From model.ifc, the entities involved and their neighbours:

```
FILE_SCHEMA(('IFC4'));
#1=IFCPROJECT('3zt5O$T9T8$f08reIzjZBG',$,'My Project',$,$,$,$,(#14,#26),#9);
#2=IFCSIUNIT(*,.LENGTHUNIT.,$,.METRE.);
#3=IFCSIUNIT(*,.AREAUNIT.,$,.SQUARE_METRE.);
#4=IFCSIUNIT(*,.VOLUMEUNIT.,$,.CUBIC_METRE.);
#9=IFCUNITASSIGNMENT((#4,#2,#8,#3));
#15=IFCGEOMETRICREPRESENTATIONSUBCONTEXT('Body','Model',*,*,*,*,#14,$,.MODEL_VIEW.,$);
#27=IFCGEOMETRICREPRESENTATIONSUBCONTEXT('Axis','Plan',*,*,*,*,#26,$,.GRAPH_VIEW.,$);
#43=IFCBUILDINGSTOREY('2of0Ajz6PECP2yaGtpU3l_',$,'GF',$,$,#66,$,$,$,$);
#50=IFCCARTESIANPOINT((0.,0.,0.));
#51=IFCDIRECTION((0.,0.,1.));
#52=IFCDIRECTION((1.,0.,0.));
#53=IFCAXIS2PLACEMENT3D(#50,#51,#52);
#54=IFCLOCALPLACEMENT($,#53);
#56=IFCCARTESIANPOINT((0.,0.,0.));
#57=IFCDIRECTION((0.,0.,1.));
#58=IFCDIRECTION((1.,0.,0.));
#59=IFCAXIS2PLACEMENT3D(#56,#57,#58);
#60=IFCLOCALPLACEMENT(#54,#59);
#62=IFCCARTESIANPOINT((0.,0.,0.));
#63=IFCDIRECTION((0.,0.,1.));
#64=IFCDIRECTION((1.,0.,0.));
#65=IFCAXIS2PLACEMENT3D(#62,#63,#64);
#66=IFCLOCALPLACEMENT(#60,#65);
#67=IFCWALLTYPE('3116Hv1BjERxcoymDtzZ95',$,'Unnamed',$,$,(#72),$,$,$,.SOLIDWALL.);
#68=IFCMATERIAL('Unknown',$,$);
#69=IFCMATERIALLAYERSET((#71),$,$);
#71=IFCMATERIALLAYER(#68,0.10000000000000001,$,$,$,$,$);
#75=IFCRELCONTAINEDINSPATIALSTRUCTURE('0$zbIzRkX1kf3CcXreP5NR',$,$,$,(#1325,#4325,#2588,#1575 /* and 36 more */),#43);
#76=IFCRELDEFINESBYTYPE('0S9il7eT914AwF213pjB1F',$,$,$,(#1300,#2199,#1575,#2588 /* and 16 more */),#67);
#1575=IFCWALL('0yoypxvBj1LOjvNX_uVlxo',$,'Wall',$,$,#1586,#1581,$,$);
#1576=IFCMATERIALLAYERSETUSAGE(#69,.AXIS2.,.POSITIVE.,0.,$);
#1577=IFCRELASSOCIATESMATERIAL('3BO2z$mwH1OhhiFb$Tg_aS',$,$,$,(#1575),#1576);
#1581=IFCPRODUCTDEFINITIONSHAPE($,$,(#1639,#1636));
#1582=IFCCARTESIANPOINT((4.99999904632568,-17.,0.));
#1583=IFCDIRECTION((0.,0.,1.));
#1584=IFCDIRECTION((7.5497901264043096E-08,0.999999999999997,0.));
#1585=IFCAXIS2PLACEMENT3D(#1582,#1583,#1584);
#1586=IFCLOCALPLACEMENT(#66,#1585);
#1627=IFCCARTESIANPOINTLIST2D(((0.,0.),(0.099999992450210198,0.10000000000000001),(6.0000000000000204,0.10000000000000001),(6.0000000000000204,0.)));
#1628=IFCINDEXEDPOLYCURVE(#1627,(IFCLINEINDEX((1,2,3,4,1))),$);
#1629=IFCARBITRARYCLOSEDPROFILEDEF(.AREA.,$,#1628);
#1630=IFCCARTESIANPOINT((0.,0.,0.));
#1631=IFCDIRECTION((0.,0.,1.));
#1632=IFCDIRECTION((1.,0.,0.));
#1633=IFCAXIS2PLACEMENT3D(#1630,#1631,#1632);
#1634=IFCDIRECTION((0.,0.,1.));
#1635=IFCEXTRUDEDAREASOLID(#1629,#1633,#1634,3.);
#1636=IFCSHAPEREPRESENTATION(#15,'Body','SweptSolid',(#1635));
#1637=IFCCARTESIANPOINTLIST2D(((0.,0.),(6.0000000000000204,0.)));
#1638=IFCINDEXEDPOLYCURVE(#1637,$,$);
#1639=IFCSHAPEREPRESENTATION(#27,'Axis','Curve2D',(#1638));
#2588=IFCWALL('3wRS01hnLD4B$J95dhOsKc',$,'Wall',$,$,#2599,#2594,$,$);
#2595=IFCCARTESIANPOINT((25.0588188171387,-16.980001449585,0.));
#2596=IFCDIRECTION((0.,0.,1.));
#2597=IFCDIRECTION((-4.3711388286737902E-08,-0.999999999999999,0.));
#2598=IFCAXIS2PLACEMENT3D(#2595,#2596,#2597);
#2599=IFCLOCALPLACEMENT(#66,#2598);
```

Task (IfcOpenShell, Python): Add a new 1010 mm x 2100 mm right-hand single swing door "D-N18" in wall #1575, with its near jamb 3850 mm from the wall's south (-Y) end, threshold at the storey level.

```python
import numpy as np
import ifcopenshell
import ifcopenshell.api.feature
import ifcopenshell.api.geometry
import ifcopenshell.api.root
import ifcopenshell.api.spatial
import ifcopenshell.geom
import ifcopenshell.util.element
import ifcopenshell.util.placement
import ifcopenshell.util.representation
import ifcopenshell.util.shape
import ifcopenshell.util.unit

model = ifcopenshell.open("model.ifc")
unit_scale = ifcopenshell.util.unit.calculate_unit_scale(model)
settings = ifcopenshell.geom.settings()


def volume(element):
    """Net volume in cubic metres, openings subtracted."""
    shape = ifcopenshell.geom.create_shape(settings, element)
    return ifcopenshell.util.shape.get_volume(shape.geometry)


wall = model.by_id(1575)
storey = ifcopenshell.util.element.get_container(wall, ifc_class="IfcBuildingStorey")
context = ifcopenshell.util.representation.get_context(model, "Model", "Body", "MODEL_VIEW")
before = volume(wall)

width, height, from_end, sill = 1.01, 2.1, 3.85, 0.0  # metres

# The wall runs along its own X axis, and the end named is its -X end.
wall_shape = ifcopenshell.geom.create_shape(settings, wall)
x, y, z = ifcopenshell.util.shape.get_vertices(wall_shape.geometry).T
start = x.min() + from_end
face, thickness = float(y.min()), float(y.max() - y.min())
wall_matrix = ifcopenshell.util.placement.get_local_placement(wall.ObjectPlacement)
level = ifcopenshell.util.placement.get_local_placement(storey.ObjectPlacement)[2, 3]


def in_wall(x, y):
    """Placement at x, y metres in the wall's axes, at sill height."""
    matrix = wall_matrix.copy()
    matrix[:, 3] = wall_matrix @ np.array([x / unit_scale, y / unit_scale, 0.0, 1.0])
    matrix[2, 3] = level + sill / unit_scale
    return matrix


# Opening: a box that overshoots both wall faces by 50 mm.
opening = ifcopenshell.api.root.create_entity(model, ifc_class="IfcOpeningElement", predefined_type="OPENING")
box = ifcopenshell.api.geometry.add_wall_representation(
    model, context=context, length=width, height=height, thickness=thickness + 0.1
)
ifcopenshell.api.geometry.assign_representation(model, product=opening, representation=box)
ifcopenshell.api.geometry.edit_object_placement(model, product=opening, matrix=in_wall(start, face - 0.05), is_si=False)
ifcopenshell.api.feature.add_feature(model, feature=opening, element=wall)

door = ifcopenshell.api.root.create_entity(model, ifc_class="IfcDoor", name="D-N18", predefined_type="DOOR")
door.OverallWidth, door.OverallHeight = width / unit_scale, height / unit_scale
door.OperationType = "SINGLE_SWING_RIGHT"
body = ifcopenshell.api.geometry.add_door_representation(
    model,
    context=context,
    overall_width=door.OverallWidth,
    overall_height=door.OverallHeight,
    operation_type="SINGLE_SWING_RIGHT",
    lining_properties={"LiningDepth": thickness / unit_scale, "ThresholdDepth": thickness / unit_scale},
)
ifcopenshell.api.geometry.assign_representation(model, product=door, representation=body)
ifcopenshell.api.spatial.assign_container(model, products=[door], relating_structure=storey)
ifcopenshell.api.feature.add_filling(model, opening=opening, element=door)

# The lining spans the wall, so the door starts at the wall face.
ifcopenshell.api.geometry.edit_object_placement(model, product=door, matrix=in_wall(start, face), is_si=False)

after = volume(wall)

print(f"wall volume {before:.3f} -> {after:.3f} m3")

model.write("model_edited.ifc")
```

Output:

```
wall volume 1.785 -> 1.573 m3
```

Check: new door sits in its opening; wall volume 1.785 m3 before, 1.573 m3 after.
